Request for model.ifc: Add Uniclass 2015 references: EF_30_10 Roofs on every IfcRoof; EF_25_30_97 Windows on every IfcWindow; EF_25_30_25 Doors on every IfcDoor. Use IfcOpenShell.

First a look at what the model holds.

```python
import ifcopenshell

model = ifcopenshell.open("model.ifc")
print(model.schema)
print("classifications:", [c.Name for c in model.by_type("IfcClassification")])
for ifc_class in ("IfcDoor", "IfcRoof", "IfcStair", "IfcWall", "IfcWindow"):
    print(ifc_class, len(model.by_type(ifc_class)))
```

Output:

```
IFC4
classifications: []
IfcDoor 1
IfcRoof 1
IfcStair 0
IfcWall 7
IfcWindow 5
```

```python
import ifcopenshell
import ifcopenshell.api.classification

model = ifcopenshell.open("model.ifc")

system = ifcopenshell.api.classification.add_classification(model, classification="Uniclass 2015")

codes = {
    "IfcRoof": ("EF_30_10", "Roofs"),
    "IfcWindow": ("EF_25_30_97", "Windows"),
    "IfcDoor": ("EF_25_30_25", "Doors"),
}
for ifc_class, (code, name) in codes.items():
    products = model.by_type(ifc_class)
    ifcopenshell.api.classification.add_reference(
        model, products=products, classification=system, identification=code, name=name
    )
    print(code, len(products))

model.write("model_edited.ifc")
```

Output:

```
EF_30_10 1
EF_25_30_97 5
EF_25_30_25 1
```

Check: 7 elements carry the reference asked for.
